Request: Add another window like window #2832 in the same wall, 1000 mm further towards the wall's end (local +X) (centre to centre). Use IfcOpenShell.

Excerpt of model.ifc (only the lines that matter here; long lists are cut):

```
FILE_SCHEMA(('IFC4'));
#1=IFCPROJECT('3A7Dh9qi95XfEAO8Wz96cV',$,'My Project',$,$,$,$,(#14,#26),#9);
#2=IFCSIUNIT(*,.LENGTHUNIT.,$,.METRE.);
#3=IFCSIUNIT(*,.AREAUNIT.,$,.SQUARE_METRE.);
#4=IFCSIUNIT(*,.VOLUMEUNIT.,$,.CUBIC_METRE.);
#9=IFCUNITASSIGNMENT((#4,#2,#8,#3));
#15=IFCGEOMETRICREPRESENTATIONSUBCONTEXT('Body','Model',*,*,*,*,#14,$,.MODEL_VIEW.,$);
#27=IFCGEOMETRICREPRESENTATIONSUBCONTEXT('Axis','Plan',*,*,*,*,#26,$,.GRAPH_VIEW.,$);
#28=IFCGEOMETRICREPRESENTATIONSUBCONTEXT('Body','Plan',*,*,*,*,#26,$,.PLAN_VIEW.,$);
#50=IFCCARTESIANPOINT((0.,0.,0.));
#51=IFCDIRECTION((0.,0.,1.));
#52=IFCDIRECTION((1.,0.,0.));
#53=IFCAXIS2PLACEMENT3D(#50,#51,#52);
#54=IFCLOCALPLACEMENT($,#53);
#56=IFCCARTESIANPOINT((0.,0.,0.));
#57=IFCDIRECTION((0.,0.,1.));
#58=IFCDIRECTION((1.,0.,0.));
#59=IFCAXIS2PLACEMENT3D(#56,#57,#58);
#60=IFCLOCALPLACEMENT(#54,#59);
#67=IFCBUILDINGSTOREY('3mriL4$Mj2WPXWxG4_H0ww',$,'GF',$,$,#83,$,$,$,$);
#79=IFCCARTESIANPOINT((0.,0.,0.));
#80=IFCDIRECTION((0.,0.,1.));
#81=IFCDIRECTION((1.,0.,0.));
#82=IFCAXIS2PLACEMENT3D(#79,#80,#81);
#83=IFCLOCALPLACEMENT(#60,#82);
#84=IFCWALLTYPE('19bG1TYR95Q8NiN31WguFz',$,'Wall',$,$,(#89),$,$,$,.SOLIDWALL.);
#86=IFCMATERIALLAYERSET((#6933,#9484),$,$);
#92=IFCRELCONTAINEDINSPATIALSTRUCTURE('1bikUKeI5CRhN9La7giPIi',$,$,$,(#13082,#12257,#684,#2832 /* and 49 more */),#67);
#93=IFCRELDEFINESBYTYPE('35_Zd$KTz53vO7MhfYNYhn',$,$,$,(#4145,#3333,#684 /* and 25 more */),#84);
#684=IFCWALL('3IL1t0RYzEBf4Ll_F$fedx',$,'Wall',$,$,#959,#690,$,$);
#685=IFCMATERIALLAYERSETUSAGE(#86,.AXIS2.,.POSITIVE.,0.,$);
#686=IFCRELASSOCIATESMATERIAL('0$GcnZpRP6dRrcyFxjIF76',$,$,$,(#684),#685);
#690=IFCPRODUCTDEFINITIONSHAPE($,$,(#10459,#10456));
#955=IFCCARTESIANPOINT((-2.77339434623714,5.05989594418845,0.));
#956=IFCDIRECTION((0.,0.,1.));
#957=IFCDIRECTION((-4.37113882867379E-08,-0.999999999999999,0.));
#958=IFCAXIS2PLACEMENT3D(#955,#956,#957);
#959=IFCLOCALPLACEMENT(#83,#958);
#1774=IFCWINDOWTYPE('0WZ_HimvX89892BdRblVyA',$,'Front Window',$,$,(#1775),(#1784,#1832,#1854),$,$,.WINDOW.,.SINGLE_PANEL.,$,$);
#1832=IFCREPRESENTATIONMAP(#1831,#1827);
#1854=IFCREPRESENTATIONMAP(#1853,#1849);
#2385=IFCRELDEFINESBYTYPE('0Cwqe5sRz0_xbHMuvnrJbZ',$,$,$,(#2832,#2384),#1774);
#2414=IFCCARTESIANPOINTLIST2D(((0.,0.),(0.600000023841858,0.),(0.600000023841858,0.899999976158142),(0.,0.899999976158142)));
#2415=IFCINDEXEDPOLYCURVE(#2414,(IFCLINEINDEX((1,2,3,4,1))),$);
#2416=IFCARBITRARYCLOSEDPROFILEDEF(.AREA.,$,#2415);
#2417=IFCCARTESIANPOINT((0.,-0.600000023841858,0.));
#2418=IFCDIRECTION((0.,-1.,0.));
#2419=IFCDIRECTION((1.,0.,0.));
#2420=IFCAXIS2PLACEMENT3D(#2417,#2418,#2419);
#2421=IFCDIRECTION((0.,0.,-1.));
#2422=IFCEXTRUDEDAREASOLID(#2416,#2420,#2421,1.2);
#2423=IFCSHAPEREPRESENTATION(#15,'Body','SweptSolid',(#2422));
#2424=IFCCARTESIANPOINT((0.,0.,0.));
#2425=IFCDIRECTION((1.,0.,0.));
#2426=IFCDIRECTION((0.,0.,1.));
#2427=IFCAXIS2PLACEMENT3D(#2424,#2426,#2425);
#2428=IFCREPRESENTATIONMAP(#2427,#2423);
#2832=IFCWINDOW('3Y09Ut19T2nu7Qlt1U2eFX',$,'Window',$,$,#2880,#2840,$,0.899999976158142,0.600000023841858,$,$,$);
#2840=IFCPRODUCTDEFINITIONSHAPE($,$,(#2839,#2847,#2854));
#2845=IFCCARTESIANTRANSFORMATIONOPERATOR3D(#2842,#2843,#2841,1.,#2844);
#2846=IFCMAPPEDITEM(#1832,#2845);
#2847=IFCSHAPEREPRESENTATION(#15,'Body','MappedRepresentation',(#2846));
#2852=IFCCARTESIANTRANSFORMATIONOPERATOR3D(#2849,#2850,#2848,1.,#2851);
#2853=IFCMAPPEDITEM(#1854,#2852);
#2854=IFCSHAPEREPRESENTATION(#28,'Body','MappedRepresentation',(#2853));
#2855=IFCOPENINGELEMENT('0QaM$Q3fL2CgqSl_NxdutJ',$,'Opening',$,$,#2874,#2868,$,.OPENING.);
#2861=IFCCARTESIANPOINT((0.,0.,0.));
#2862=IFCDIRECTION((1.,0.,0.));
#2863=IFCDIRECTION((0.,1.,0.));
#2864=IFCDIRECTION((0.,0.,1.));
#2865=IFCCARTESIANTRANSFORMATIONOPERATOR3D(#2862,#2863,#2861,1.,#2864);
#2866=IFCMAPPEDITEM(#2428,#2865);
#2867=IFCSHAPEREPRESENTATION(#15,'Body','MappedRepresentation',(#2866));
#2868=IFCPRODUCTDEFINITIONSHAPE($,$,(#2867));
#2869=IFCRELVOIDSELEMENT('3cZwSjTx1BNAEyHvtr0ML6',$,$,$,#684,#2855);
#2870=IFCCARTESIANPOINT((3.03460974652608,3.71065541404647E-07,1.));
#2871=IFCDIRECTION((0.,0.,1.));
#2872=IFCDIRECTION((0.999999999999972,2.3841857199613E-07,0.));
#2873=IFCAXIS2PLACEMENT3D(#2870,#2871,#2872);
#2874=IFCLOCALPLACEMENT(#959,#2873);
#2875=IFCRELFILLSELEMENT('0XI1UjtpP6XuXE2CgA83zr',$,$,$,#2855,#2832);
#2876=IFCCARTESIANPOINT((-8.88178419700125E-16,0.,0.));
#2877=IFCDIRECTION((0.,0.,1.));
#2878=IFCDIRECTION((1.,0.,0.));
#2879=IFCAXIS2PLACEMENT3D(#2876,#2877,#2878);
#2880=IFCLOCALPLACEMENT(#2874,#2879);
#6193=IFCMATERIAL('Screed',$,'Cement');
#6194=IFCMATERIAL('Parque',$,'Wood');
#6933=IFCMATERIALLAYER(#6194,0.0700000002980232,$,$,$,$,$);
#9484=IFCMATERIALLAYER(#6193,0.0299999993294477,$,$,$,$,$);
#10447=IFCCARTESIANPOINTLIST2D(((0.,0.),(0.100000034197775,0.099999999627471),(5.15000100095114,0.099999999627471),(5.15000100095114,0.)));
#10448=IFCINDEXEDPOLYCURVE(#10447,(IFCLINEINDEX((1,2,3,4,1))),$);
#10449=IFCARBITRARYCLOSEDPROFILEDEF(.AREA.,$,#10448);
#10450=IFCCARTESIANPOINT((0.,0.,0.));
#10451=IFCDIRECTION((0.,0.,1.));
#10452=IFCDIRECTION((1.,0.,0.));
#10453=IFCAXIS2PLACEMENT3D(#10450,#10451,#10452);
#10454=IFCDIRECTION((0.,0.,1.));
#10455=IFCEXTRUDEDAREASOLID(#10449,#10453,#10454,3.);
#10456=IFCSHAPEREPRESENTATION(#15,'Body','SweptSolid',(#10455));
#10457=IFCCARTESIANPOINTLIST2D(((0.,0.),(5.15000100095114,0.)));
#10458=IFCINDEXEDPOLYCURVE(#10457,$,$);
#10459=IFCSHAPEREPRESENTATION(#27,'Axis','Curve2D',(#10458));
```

```python
import ifcopenshell
import ifcopenshell.api.feature
import ifcopenshell.api.geometry
import ifcopenshell.api.root
import ifcopenshell.geom
import ifcopenshell.util.element
import ifcopenshell.util.placement
import ifcopenshell.util.shape

model = ifcopenshell.open("model.ifc")
settings = ifcopenshell.geom.settings()


def volume(element):
    """Net volume in cubic metres, openings subtracted."""
    shape = ifcopenshell.geom.create_shape(settings, element)
    return ifcopenshell.util.shape.get_volume(shape.geometry)


window = model.by_guid("3Y09Ut19T2nu7Qlt1U2eFX")
opening = window.FillsVoids[0].RelatingOpeningElement
wall = opening.VoidsElements[0].RelatingBuildingElement
before = volume(wall)
shift = ifcopenshell.util.placement.get_local_placement(wall.ObjectPlacement)[:3, 0] * 1.0

# copy_class copies the void relationship, type, container and properties, but no geometry.
new_opening = ifcopenshell.api.root.copy_class(model, product=opening)
new_opening.Representation = ifcopenshell.util.element.copy_deep(
    model, opening.Representation, exclude=["IfcGeometricRepresentationContext", "IfcRepresentationMap"]
)
new_window = ifcopenshell.api.root.copy_class(model, product=window)
new_window.Representation = ifcopenshell.util.element.copy_deep(
    model, window.Representation, exclude=["IfcGeometricRepresentationContext", "IfcRepresentationMap"]
)
ifcopenshell.api.feature.add_filling(model, opening=new_opening, element=new_window)

for old, new in ((opening, new_opening), (window, new_window)):
    matrix = ifcopenshell.util.placement.get_local_placement(old.ObjectPlacement)
    matrix[:3, 3] += shift
    ifcopenshell.api.geometry.edit_object_placement(model, product=new, matrix=matrix, is_si=False)

after = volume(wall)

print(f"wall volume {before:.3f} -> {after:.3f} m3")

model.write("model-out.ifc")
```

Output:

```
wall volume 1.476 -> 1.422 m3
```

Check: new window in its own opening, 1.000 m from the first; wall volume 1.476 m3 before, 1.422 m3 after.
